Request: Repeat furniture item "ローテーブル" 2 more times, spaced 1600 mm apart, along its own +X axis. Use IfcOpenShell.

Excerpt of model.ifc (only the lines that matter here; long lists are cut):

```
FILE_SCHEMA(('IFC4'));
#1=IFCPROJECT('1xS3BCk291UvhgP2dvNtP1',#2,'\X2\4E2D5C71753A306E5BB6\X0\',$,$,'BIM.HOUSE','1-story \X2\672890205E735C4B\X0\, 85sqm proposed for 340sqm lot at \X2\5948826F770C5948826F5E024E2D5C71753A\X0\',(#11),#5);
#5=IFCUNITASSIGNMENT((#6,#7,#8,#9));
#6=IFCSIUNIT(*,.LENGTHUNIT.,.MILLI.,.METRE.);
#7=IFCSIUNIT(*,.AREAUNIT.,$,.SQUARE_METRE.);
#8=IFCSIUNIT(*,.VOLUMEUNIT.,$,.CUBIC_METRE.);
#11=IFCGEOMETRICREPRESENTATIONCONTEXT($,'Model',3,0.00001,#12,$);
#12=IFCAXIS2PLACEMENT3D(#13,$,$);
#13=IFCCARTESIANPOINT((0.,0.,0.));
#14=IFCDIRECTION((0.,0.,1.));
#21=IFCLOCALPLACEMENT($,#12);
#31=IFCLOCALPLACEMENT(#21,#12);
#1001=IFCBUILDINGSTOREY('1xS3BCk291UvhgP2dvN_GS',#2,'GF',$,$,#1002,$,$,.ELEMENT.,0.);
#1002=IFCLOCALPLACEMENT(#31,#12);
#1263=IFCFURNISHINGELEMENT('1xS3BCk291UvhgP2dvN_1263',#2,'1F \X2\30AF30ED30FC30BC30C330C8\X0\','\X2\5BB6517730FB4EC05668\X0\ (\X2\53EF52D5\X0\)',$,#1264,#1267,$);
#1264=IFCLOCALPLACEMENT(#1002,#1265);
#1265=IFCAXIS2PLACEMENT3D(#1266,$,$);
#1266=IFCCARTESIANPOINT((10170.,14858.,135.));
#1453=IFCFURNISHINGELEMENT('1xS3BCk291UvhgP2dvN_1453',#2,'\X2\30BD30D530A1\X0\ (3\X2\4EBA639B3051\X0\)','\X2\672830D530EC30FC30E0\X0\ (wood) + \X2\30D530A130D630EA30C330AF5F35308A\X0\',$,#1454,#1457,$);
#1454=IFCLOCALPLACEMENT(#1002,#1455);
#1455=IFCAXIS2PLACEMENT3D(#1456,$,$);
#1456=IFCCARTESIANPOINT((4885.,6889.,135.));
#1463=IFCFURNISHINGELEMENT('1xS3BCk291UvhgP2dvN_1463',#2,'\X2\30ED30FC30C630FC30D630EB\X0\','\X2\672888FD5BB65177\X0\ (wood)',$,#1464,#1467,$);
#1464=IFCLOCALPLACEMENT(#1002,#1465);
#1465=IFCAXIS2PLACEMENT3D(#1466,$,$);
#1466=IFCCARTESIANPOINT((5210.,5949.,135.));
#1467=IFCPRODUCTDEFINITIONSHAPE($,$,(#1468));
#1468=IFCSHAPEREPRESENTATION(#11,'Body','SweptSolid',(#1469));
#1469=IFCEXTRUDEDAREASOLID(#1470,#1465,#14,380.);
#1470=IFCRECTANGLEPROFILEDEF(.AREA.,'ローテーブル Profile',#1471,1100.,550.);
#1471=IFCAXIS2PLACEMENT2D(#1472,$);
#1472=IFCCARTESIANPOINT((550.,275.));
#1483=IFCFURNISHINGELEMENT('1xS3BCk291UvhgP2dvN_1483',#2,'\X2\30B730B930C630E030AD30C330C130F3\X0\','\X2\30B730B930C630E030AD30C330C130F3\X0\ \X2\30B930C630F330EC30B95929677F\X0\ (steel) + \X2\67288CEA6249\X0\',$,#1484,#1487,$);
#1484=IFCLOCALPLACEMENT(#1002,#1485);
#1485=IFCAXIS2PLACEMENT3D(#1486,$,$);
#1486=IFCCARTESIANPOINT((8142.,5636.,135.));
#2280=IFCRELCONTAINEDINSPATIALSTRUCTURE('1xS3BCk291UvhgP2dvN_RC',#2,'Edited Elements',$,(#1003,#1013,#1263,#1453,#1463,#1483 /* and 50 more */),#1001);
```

```python
import ifcopenshell
import ifcopenshell.api.geometry
import ifcopenshell.api.root
import ifcopenshell.util.element
import ifcopenshell.util.placement
import ifcopenshell.util.unit

model = ifcopenshell.open("model.ifc")
unit_scale = ifcopenshell.util.unit.calculate_unit_scale(model)


def reuse_history(source, copy):
    """copy_class also copies each property set's owner history, people and application; keep the originals."""
    for rel in copy.IsDefinedBy:
        if rel.is_a("IfcRelDefinesByProperties") and (history := rel.RelatingPropertyDefinition.OwnerHistory):
            rel.RelatingPropertyDefinition.OwnerHistory = source.OwnerHistory
            ifcopenshell.util.element.remove_deep2(model, history)


source = model.by_guid("1xS3BCk291UvhgP2dvN_1463")
base = ifcopenshell.util.placement.get_local_placement(source.ObjectPlacement)
step = base[:3, 0] * 1.6 / unit_scale

for i in range(1, 3):
    copy = ifcopenshell.api.root.copy_class(model, product=source)
    copy.Representation = ifcopenshell.util.element.copy_deep(
        model, source.Representation, exclude=["IfcGeometricRepresentationContext", "IfcRepresentationMap"]
    )
    reuse_history(source, copy)
    matrix = base.copy()
    matrix[:3, 3] += i * step
    print("added at", matrix[:3, 3].round(3) + 0.0)
    ifcopenshell.api.geometry.edit_object_placement(model, product=copy, matrix=matrix, is_si=False)

model.write("model_edited.ifc")
```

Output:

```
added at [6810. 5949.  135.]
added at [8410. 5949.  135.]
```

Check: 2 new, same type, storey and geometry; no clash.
